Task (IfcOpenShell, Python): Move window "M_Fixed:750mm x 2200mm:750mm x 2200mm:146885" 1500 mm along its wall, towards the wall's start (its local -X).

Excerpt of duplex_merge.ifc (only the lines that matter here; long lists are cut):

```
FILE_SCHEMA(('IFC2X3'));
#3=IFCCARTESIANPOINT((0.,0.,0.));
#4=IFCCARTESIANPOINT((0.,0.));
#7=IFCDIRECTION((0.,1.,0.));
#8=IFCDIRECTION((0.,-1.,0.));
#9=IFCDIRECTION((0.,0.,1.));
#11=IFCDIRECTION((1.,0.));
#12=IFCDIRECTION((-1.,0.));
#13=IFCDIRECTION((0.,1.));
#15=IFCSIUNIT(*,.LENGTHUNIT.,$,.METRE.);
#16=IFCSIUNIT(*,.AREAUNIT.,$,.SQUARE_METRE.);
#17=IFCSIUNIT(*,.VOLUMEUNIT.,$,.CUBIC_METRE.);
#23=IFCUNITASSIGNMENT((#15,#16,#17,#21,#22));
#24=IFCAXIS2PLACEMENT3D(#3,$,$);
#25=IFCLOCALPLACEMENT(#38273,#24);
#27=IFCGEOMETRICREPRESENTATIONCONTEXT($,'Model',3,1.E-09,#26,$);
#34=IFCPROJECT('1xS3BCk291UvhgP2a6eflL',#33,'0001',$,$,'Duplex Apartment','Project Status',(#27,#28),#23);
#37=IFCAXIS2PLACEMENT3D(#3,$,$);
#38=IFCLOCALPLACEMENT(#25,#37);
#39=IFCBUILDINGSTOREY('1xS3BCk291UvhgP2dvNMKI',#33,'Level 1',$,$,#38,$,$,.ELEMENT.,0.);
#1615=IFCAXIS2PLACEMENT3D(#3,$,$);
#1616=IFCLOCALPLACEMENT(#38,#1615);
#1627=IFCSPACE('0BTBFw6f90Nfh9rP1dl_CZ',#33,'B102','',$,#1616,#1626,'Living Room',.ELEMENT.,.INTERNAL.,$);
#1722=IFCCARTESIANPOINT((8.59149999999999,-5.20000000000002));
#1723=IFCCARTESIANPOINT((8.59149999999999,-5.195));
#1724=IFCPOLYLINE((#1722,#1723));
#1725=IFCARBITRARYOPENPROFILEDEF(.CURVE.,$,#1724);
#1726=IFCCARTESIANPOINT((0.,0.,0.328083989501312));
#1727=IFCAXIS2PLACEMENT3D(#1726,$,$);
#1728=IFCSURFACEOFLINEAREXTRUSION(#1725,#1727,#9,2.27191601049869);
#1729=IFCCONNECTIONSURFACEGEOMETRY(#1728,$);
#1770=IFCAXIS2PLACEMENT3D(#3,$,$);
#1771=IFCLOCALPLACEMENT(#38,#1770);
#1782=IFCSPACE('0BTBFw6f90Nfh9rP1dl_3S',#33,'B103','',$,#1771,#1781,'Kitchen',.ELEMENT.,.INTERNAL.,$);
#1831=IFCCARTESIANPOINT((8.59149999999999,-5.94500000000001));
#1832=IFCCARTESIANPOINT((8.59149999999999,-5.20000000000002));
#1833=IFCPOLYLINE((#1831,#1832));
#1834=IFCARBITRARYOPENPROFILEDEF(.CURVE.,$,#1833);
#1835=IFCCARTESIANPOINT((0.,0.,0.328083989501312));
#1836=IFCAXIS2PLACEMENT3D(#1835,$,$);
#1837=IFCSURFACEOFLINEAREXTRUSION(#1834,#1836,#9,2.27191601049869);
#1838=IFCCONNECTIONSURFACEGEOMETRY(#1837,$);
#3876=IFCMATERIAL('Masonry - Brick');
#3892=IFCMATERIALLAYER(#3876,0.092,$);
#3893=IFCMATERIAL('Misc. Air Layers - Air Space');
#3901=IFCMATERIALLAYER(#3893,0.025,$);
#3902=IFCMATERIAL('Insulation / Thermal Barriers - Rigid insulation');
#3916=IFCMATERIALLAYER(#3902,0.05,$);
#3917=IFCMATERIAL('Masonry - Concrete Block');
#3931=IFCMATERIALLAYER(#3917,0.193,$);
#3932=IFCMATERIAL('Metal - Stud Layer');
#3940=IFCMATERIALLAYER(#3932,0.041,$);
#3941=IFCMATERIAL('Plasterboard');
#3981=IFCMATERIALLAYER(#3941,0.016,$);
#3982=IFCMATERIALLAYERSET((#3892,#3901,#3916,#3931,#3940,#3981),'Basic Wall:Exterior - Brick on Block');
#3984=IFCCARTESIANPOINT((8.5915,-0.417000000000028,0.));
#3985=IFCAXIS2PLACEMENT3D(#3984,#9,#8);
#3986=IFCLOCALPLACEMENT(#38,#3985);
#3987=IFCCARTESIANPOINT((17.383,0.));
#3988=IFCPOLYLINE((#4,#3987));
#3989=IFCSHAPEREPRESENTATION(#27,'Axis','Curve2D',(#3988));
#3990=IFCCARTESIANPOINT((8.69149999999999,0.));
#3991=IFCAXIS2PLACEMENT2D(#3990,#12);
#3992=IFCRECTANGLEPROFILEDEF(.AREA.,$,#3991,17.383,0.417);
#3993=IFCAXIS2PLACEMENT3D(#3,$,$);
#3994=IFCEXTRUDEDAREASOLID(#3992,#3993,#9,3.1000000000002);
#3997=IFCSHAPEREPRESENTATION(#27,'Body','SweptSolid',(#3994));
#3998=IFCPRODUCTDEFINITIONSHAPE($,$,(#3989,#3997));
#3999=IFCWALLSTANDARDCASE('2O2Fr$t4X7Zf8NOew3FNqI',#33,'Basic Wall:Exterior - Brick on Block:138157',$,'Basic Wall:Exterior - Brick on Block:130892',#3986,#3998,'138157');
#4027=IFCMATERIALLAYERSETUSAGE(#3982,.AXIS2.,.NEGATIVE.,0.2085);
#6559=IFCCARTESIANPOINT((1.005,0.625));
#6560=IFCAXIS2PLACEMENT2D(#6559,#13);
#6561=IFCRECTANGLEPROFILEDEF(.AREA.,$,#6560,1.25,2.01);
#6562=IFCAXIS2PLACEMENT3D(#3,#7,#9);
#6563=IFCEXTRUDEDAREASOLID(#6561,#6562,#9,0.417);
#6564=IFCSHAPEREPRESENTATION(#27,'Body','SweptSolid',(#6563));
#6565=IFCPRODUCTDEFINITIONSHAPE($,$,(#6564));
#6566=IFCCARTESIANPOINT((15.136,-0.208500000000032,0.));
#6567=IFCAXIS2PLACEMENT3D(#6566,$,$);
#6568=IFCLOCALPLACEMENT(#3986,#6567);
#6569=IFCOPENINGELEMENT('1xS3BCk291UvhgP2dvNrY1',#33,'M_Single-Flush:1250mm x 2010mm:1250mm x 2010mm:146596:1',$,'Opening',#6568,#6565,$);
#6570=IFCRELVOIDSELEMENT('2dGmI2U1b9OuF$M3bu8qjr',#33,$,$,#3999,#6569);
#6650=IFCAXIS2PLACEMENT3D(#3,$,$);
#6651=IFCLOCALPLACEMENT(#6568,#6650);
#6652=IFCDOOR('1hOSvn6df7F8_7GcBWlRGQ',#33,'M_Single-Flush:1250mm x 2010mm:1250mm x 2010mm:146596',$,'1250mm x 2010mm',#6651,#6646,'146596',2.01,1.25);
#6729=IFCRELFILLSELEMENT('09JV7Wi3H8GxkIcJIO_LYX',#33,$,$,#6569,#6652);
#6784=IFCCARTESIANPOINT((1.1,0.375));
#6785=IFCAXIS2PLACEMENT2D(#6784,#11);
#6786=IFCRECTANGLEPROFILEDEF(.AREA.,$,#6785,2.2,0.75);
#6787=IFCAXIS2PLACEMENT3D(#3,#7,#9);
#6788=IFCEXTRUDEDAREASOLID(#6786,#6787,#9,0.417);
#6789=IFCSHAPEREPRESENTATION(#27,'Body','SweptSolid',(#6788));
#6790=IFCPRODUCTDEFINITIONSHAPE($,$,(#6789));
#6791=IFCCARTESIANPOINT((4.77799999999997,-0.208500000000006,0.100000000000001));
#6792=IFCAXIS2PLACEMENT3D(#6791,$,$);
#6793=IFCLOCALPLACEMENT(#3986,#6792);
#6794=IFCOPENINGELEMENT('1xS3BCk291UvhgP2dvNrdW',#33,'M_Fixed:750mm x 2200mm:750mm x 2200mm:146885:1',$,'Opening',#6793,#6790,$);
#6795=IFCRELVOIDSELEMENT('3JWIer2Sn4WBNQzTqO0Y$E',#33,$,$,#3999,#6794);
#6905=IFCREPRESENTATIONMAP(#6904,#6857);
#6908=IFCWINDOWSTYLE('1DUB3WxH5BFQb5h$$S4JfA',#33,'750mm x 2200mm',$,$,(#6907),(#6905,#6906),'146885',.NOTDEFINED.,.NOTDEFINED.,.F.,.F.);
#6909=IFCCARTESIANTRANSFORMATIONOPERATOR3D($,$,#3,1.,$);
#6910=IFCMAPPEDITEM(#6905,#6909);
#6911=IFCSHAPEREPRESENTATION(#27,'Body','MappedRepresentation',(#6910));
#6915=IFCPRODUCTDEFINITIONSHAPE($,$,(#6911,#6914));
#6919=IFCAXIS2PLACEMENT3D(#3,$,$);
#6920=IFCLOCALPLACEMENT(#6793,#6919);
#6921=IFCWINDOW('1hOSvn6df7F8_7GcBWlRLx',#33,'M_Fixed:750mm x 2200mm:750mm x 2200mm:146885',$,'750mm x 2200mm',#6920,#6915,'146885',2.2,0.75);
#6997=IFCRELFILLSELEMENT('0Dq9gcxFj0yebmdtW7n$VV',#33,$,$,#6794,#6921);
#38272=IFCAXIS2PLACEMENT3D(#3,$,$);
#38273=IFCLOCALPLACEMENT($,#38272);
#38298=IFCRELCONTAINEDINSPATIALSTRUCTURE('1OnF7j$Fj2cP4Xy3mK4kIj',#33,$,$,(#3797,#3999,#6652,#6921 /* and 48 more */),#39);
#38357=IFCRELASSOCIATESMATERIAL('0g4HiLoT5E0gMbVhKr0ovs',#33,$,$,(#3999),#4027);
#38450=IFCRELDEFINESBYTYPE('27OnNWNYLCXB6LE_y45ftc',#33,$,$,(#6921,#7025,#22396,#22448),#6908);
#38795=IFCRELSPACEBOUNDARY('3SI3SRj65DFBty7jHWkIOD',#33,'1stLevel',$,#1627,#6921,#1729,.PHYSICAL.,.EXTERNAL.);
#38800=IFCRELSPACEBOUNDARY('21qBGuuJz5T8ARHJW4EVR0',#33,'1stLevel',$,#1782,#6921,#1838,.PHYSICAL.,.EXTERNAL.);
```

```python
import numpy as np
import ifcopenshell
import ifcopenshell.api.geometry
import ifcopenshell.util.placement
import ifcopenshell.util.unit

model = ifcopenshell.open("duplex_merge.ifc")
unit_scale = ifcopenshell.util.unit.calculate_unit_scale(model)

window = model.by_id(6921)
opening = window.FillsVoids[0].RelatingOpeningElement
wall = opening.VoidsElements[0].RelatingBuildingElement

wall_matrix = ifcopenshell.util.placement.get_local_placement(wall.ObjectPlacement)
shift = wall_matrix[:3, 0] * -1.5 / unit_scale
before = ifcopenshell.util.placement.get_local_placement(window.ObjectPlacement)[:3, 3].copy()

# The window is placed relative to its opening, so it follows when the opening moves.
matrix = ifcopenshell.util.placement.get_local_placement(opening.ObjectPlacement)
matrix[:3, 3] += shift
ifcopenshell.api.geometry.edit_object_placement(
    model, product=opening, matrix=matrix, is_si=False, should_transform_children=True
)

# Space boundary surfaces are stored in each space's coordinates; move them too.
for rel in window.ProvidesBoundaries:
    if not rel.ConnectionGeometry:
        continue
    surface = rel.ConnectionGeometry.SurfaceOnRelatingElement
    space_matrix = ifcopenshell.util.placement.get_local_placement(rel.RelatingSpace.ObjectPlacement)
    point = np.array(surface.Position.Location.Coordinates) + space_matrix[:3, :3].T @ shift
    surface.Position = model.createIfcAxis2Placement3D(
        model.createIfcCartesianPoint(point.tolist()), surface.Position.Axis, surface.Position.RefDirection
    )

after = ifcopenshell.util.placement.get_local_placement(window.ObjectPlacement)[:3, 3]
print("window moved by", (after - before).round(3) + 0.0)

model.write("duplex_merge_rev.ifc")
```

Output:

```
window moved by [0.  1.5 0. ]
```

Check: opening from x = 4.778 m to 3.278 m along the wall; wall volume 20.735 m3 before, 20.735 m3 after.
